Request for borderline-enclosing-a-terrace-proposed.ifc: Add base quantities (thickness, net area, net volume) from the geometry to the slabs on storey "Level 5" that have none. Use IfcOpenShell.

First a look at what the model holds.

```python
import ifcopenshell
import ifcopenshell.util.element
import ifcopenshell.util.unit

model = ifcopenshell.open("borderline-enclosing-a-terrace-proposed.ifc")
print(model.schema)
for unit_type in ("LENGTHUNIT", "AREAUNIT", "VOLUMEUNIT"):
    print(unit_type, ifcopenshell.util.unit.calculate_unit_scale(model, unit_type))
storey = next(s for s in model.by_type("IfcBuildingStorey") if s.Name == "Level 5")
slabs = [e for e in ifcopenshell.util.element.get_decomposition(storey) if e.is_a("IfcSlab")]
for e in sorted(slabs, key=lambda e: e.id()):
    print(e.id(), e.is_a(), e.Name, list(ifcopenshell.util.element.get_psets(e, qtos_only=True)), sep=" | ")
```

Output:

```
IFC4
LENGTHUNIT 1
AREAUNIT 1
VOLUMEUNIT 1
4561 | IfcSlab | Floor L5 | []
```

```python
import ifcopenshell
import ifcopenshell.api.pset
import ifcopenshell.geom
import ifcopenshell.util.element
import ifcopenshell.util.shape
import ifcopenshell.util.unit

model = ifcopenshell.open("borderline-enclosing-a-terrace-proposed.ifc")
unit_scale = ifcopenshell.util.unit.calculate_unit_scale(model)
area_scale = ifcopenshell.util.unit.calculate_unit_scale(model, "AREAUNIT")
volume_scale = ifcopenshell.util.unit.calculate_unit_scale(model, "VOLUMEUNIT")
settings = ifcopenshell.geom.settings()

storey = next(s for s in model.by_type("IfcBuildingStorey") if s.Name == "Level 5")
slabs = [e for e in ifcopenshell.util.element.get_decomposition(storey) if e.is_a("IfcSlab")]

for e in sorted(slabs, key=lambda e: e.id()):
    if ifcopenshell.util.element.get_psets(e, qtos_only=True, should_inherit=False):
        continue
    # Geometry comes back in metres, in the element's own axes.
    shape = ifcopenshell.geom.create_shape(settings, e)
    values = {
        "Width": ifcopenshell.util.shape.get_z(shape.geometry) / unit_scale,
        "NetArea": ifcopenshell.util.shape.get_footprint_area(shape.geometry) / area_scale,
        "NetVolume": ifcopenshell.util.shape.get_volume(shape.geometry) / volume_scale,
    }
    qto = ifcopenshell.api.pset.add_qto(model, product=e, name="Qto_SlabBaseQuantities")
    ifcopenshell.api.pset.edit_qto(model, qto=qto, properties=values)
    print(e.id(), {k: round(v, 3) for k, v in values.items()})

model.write("borderline-enclosing-a-terrace-proposed_rev.ifc")
```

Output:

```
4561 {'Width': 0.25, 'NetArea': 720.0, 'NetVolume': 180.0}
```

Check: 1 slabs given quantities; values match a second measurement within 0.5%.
